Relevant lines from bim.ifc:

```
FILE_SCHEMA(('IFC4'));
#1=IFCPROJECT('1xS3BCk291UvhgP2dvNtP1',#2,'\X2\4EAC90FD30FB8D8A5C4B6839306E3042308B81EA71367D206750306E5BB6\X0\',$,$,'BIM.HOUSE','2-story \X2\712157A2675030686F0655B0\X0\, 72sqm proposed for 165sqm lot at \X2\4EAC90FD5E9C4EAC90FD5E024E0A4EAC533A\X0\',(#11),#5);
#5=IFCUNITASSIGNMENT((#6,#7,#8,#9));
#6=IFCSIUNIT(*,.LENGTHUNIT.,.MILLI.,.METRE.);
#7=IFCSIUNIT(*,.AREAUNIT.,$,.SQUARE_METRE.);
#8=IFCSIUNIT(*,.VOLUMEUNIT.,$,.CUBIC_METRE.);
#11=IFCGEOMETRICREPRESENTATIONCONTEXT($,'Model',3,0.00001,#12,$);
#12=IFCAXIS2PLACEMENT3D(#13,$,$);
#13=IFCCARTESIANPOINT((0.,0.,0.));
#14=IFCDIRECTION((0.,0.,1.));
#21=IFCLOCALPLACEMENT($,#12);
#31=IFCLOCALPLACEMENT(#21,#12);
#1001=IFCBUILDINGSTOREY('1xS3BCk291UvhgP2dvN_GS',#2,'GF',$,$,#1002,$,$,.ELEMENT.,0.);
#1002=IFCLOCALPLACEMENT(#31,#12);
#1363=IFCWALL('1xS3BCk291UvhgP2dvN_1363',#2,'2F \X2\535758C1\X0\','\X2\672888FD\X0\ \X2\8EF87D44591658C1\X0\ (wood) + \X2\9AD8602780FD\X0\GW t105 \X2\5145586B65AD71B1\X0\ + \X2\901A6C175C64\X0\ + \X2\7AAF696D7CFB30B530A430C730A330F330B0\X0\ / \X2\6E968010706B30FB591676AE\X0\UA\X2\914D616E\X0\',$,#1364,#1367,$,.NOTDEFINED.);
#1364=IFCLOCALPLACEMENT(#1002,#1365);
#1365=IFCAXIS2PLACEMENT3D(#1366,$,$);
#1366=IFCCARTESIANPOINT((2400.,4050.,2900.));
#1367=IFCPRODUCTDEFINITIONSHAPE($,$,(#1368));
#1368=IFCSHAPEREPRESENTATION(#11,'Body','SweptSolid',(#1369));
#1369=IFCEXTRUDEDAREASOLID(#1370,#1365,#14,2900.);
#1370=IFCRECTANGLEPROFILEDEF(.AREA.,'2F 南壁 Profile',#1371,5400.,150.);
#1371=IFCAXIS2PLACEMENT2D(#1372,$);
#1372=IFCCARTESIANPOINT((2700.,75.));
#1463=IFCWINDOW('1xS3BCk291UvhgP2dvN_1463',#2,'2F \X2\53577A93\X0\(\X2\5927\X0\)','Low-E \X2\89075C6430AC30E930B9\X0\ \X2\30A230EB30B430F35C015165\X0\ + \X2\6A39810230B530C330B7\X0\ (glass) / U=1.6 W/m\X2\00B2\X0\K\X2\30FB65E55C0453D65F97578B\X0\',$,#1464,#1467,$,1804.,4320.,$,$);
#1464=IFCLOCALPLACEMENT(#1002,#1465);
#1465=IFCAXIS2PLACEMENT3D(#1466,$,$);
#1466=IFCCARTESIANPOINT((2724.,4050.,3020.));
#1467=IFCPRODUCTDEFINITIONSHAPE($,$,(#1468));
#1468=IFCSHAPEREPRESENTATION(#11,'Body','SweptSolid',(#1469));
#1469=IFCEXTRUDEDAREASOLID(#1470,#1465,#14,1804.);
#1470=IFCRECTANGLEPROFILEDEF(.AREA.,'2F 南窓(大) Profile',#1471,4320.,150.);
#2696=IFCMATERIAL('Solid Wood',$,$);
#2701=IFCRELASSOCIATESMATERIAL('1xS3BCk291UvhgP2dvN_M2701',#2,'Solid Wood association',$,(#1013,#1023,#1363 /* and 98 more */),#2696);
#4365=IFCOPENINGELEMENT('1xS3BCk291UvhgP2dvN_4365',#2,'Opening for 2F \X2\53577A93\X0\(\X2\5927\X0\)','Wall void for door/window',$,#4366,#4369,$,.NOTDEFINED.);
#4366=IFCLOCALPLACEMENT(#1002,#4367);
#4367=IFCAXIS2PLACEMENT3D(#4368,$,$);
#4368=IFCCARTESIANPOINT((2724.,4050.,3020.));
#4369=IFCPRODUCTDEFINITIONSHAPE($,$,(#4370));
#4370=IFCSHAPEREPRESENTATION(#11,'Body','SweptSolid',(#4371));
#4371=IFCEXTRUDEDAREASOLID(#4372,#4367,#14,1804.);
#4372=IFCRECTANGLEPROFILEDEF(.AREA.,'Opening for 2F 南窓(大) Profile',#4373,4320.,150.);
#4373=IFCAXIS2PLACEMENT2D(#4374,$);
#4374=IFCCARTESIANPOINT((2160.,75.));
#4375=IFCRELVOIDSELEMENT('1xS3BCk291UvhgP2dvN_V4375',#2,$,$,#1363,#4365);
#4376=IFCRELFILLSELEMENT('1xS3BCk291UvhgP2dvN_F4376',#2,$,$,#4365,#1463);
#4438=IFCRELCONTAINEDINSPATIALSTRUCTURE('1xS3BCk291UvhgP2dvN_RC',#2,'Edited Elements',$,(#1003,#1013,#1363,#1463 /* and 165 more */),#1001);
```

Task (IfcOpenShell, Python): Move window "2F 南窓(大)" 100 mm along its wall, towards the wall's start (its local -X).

```python
import ifcopenshell
import ifcopenshell.api.geometry
import ifcopenshell.util.placement

model = ifcopenshell.open("bim.ifc")

window = model.by_id(1463)
opening = window.FillsVoids[0].RelatingOpeningElement
wall = opening.VoidsElements[0].RelatingBuildingElement

wall_matrix = ifcopenshell.util.placement.get_local_placement(wall.ObjectPlacement)
shift = wall_matrix[:3, 0] * -100.0
before = ifcopenshell.util.placement.get_local_placement(window.ObjectPlacement)[:3, 3].copy()

# The window is not placed relative to its opening, so move both.
for product in (opening, window):
    matrix = ifcopenshell.util.placement.get_local_placement(product.ObjectPlacement)
    matrix[:3, 3] += shift
    ifcopenshell.api.geometry.edit_object_placement(model, product=product, matrix=matrix, is_si=False)

after = ifcopenshell.util.placement.get_local_placement(window.ObjectPlacement)[:3, 3]
print("window moved by", (after - before).round(3) + 0.0)

model.write("bim_edited.ifc")
```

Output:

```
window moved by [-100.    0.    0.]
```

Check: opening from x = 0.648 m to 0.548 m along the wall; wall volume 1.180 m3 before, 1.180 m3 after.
